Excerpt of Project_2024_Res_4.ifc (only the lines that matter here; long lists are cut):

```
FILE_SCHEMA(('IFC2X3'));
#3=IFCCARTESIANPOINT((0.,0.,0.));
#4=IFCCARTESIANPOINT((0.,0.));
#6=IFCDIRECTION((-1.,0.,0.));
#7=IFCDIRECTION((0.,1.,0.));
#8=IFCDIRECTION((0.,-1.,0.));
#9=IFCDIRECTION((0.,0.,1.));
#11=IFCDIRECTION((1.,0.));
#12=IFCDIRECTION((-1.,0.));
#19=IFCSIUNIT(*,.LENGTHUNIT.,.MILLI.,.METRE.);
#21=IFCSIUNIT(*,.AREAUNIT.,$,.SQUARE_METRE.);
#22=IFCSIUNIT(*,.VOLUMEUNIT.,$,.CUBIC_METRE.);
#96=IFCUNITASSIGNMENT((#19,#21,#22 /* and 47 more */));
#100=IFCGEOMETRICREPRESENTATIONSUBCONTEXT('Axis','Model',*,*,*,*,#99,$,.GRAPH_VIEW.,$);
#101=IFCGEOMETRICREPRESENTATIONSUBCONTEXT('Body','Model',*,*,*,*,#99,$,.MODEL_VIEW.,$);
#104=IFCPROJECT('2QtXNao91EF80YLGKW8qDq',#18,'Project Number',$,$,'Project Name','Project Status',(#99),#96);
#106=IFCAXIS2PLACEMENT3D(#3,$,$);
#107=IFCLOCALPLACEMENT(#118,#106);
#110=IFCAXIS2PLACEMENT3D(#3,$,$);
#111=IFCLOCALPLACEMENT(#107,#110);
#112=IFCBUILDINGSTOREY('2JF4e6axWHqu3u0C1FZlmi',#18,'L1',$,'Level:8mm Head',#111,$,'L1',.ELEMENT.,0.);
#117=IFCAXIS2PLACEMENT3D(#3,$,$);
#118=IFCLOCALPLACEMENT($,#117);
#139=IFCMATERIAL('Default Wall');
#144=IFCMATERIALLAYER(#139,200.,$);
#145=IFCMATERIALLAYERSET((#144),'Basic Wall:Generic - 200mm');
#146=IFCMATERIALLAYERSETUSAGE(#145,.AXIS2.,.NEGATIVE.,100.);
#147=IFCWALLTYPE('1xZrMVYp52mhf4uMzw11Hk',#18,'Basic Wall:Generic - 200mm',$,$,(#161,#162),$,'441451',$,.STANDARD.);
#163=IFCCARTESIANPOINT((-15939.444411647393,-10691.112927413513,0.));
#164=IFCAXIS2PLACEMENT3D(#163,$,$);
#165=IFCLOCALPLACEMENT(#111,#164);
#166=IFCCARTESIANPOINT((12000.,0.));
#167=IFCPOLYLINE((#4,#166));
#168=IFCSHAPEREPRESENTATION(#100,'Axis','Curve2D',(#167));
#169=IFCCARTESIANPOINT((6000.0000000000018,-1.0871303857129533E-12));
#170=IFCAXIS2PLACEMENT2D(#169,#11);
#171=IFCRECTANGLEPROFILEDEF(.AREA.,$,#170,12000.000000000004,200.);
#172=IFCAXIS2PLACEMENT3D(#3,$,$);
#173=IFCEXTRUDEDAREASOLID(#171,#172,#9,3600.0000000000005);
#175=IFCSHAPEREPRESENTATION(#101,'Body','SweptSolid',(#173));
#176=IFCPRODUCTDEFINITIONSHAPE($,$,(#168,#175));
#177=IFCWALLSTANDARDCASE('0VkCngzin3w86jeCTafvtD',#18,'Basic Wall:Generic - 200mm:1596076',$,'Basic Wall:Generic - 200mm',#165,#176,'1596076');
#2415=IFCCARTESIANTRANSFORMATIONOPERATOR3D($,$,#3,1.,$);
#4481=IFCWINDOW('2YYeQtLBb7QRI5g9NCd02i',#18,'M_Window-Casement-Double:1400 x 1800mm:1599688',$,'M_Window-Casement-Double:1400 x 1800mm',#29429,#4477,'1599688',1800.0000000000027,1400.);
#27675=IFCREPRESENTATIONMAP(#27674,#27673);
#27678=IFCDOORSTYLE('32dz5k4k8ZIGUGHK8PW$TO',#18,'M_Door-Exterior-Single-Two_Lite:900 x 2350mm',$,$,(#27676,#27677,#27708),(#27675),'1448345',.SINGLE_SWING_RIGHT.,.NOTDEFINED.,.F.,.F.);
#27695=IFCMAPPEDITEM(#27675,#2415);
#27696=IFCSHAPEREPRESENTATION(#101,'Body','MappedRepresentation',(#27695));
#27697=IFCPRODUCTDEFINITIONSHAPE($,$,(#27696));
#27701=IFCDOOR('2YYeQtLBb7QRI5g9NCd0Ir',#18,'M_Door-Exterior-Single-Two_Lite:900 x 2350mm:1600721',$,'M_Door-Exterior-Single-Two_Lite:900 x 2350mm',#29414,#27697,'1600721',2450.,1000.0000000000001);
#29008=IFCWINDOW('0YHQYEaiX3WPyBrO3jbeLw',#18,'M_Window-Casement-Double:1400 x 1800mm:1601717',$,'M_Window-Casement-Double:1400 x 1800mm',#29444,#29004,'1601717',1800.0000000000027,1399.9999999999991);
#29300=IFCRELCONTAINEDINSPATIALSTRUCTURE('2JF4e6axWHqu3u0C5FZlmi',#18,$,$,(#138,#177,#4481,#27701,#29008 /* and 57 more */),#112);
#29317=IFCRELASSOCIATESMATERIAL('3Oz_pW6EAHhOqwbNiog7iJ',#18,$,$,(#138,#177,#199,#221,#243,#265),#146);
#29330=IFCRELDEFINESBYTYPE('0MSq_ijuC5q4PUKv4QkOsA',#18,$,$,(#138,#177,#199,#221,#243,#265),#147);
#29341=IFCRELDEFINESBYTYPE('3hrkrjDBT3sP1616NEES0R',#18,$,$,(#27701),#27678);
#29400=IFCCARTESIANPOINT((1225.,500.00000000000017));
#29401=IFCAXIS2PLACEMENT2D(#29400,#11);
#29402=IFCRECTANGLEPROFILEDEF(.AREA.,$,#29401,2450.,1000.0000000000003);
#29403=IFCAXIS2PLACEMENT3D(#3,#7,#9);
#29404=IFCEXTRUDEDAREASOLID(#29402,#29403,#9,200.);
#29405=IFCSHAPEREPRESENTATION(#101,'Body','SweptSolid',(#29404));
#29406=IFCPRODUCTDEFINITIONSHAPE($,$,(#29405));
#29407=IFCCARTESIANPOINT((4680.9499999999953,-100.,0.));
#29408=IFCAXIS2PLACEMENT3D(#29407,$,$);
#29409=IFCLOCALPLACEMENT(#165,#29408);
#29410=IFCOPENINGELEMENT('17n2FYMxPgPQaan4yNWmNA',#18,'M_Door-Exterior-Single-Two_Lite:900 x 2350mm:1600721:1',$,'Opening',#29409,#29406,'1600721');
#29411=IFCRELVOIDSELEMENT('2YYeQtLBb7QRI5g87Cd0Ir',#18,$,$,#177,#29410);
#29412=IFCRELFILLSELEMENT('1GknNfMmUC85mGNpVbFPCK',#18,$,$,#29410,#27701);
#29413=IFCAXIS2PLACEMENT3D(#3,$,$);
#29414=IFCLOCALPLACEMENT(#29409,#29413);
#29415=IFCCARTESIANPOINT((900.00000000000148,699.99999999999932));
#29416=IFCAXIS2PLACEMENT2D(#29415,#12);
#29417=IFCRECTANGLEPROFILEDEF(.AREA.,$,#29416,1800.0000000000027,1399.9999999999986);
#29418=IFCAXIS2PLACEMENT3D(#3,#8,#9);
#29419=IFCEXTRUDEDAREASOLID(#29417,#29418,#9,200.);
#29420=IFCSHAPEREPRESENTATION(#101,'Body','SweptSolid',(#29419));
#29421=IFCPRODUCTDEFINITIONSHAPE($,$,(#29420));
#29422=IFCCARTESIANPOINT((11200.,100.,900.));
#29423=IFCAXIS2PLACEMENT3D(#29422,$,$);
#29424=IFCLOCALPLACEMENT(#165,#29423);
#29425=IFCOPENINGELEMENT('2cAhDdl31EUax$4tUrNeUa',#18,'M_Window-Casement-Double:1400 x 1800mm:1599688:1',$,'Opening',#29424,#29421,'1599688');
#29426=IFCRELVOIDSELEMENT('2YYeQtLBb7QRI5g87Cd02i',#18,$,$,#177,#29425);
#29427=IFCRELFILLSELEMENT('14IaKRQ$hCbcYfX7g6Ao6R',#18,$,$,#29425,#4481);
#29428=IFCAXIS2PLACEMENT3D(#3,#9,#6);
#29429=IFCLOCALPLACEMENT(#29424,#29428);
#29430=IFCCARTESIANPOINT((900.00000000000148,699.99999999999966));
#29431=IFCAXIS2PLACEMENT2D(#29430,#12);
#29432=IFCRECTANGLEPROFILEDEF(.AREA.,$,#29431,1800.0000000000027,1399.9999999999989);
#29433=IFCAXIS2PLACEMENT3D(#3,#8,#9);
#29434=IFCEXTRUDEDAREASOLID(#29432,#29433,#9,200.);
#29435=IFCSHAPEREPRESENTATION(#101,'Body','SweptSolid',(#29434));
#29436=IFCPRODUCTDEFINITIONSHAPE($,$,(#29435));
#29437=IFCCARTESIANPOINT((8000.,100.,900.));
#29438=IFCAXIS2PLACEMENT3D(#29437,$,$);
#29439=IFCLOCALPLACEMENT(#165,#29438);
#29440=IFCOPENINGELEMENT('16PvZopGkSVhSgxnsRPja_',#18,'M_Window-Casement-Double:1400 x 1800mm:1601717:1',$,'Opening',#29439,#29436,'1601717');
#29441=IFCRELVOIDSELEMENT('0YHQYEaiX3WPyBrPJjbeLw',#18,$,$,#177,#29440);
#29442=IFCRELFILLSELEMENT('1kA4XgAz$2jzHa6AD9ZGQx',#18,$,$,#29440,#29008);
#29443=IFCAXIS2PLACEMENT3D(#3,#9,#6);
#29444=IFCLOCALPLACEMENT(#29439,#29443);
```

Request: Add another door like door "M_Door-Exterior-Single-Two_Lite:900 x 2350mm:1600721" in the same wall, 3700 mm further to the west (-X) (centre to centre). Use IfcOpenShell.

```python
import ifcopenshell
import ifcopenshell.api.feature
import ifcopenshell.api.geometry
import ifcopenshell.api.root
import ifcopenshell.geom
import ifcopenshell.util.element
import ifcopenshell.util.placement
import ifcopenshell.util.shape

model = ifcopenshell.open("Project_2024_Res_4.ifc")
settings = ifcopenshell.geom.settings()


def volume(element):
    """Net volume in cubic metres, openings subtracted."""
    shape = ifcopenshell.geom.create_shape(settings, element)
    return ifcopenshell.util.shape.get_volume(shape.geometry)


def reuse_history(source, copy):
    """copy_class also copies each property set's owner history, people and application; keep the originals."""
    for rel in copy.IsDefinedBy:
        if rel.is_a("IfcRelDefinesByProperties") and (history := rel.RelatingPropertyDefinition.OwnerHistory):
            rel.RelatingPropertyDefinition.OwnerHistory = source.OwnerHistory
            ifcopenshell.util.element.remove_deep2(model, history)


door = model.by_guid("2YYeQtLBb7QRI5g9NCd0Ir")
opening = door.FillsVoids[0].RelatingOpeningElement
wall = opening.VoidsElements[0].RelatingBuildingElement
before = volume(wall)
shift = ifcopenshell.util.placement.get_local_placement(wall.ObjectPlacement)[:3, 0] * -3700.0

# copy_class copies the void relationship, type, container and properties, but no geometry.
new_opening = ifcopenshell.api.root.copy_class(model, product=opening)
new_opening.Representation = ifcopenshell.util.element.copy_deep(
    model, opening.Representation, exclude=["IfcGeometricRepresentationContext", "IfcRepresentationMap"]
)
new_opening.Name = "M_Door-Exterior-Single-Two_Lite:900 x 2350mm"
new_opening.Tag = None
new_door = ifcopenshell.api.root.copy_class(model, product=door)
new_door.Representation = ifcopenshell.util.element.copy_deep(
    model, door.Representation, exclude=["IfcGeometricRepresentationContext", "IfcRepresentationMap"]
)
new_door.Name = "M_Door-Exterior-Single-Two_Lite:900 x 2350mm"
new_door.Tag = None
reuse_history(door, new_door)
fills = ifcopenshell.api.feature.add_filling(model, opening=new_opening, element=new_door)
fills.OwnerHistory = new_door.OwnerHistory  # required in IFC2X3

for old, new in ((opening, new_opening), (door, new_door)):
    matrix = ifcopenshell.util.placement.get_local_placement(old.ObjectPlacement)
    matrix[:3, 3] += shift
    ifcopenshell.api.geometry.edit_object_placement(model, product=new, matrix=matrix, is_si=False)

after = volume(wall)

print(f"wall volume {before:.3f} -> {after:.3f} m3")

model.write("Project_2024_Res_4-out.ifc")
```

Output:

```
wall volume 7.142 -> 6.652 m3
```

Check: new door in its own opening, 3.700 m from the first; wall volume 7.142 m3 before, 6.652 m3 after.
